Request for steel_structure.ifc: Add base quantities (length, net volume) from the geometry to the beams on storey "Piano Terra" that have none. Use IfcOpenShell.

First a look at what the model holds.

```python
import ifcopenshell
import ifcopenshell.util.element
import ifcopenshell.util.unit

model = ifcopenshell.open("steel_structure.ifc")
print(model.schema)
for unit_type in ("LENGTHUNIT", "AREAUNIT", "VOLUMEUNIT"):
    print(unit_type, ifcopenshell.util.unit.calculate_unit_scale(model, unit_type))
storey = next(s for s in model.by_type("IfcBuildingStorey") if s.Name == "Piano Terra")
beams = [e for e in ifcopenshell.util.element.get_decomposition(storey) if e.is_a("IfcBeam")]
for e in sorted(beams, key=lambda e: e.id()):
    print(e.id(), e.is_a(), e.Name, list(ifcopenshell.util.element.get_psets(e, qtos_only=True)), sep=" | ")
```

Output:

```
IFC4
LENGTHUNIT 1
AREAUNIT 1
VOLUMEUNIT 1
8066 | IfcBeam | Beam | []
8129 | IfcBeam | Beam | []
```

```python
import ifcopenshell
import ifcopenshell.api.pset
import ifcopenshell.geom
import ifcopenshell.util.element
import ifcopenshell.util.shape
import ifcopenshell.util.unit

model = ifcopenshell.open("steel_structure.ifc")
unit_scale = ifcopenshell.util.unit.calculate_unit_scale(model)
volume_scale = ifcopenshell.util.unit.calculate_unit_scale(model, "VOLUMEUNIT")
settings = ifcopenshell.geom.settings()

storey = next(s for s in model.by_type("IfcBuildingStorey") if s.Name == "Piano Terra")
beams = [e for e in ifcopenshell.util.element.get_decomposition(storey) if e.is_a("IfcBeam")]

for e in sorted(beams, key=lambda e: e.id()):
    if ifcopenshell.util.element.get_psets(e, qtos_only=True, should_inherit=False):
        continue
    # Geometry comes back in metres, in the element's own axes.
    shape = ifcopenshell.geom.create_shape(settings, e)
    values = {
        "Length": ifcopenshell.util.shape.get_max_xyz(shape.geometry) / unit_scale,
        "NetVolume": ifcopenshell.util.shape.get_volume(shape.geometry) / volume_scale,
    }
    qto = ifcopenshell.api.pset.add_qto(model, product=e, name="Qto_BeamBaseQuantities")
    ifcopenshell.api.pset.edit_qto(model, qto=qto, properties=values)
    print(e.id(), {k: round(v, 3) for k, v in values.items()})

model.write("steel_structure_v2.ifc")
```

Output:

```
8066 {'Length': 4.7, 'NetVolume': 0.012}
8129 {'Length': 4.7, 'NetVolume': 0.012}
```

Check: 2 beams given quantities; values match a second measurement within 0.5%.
